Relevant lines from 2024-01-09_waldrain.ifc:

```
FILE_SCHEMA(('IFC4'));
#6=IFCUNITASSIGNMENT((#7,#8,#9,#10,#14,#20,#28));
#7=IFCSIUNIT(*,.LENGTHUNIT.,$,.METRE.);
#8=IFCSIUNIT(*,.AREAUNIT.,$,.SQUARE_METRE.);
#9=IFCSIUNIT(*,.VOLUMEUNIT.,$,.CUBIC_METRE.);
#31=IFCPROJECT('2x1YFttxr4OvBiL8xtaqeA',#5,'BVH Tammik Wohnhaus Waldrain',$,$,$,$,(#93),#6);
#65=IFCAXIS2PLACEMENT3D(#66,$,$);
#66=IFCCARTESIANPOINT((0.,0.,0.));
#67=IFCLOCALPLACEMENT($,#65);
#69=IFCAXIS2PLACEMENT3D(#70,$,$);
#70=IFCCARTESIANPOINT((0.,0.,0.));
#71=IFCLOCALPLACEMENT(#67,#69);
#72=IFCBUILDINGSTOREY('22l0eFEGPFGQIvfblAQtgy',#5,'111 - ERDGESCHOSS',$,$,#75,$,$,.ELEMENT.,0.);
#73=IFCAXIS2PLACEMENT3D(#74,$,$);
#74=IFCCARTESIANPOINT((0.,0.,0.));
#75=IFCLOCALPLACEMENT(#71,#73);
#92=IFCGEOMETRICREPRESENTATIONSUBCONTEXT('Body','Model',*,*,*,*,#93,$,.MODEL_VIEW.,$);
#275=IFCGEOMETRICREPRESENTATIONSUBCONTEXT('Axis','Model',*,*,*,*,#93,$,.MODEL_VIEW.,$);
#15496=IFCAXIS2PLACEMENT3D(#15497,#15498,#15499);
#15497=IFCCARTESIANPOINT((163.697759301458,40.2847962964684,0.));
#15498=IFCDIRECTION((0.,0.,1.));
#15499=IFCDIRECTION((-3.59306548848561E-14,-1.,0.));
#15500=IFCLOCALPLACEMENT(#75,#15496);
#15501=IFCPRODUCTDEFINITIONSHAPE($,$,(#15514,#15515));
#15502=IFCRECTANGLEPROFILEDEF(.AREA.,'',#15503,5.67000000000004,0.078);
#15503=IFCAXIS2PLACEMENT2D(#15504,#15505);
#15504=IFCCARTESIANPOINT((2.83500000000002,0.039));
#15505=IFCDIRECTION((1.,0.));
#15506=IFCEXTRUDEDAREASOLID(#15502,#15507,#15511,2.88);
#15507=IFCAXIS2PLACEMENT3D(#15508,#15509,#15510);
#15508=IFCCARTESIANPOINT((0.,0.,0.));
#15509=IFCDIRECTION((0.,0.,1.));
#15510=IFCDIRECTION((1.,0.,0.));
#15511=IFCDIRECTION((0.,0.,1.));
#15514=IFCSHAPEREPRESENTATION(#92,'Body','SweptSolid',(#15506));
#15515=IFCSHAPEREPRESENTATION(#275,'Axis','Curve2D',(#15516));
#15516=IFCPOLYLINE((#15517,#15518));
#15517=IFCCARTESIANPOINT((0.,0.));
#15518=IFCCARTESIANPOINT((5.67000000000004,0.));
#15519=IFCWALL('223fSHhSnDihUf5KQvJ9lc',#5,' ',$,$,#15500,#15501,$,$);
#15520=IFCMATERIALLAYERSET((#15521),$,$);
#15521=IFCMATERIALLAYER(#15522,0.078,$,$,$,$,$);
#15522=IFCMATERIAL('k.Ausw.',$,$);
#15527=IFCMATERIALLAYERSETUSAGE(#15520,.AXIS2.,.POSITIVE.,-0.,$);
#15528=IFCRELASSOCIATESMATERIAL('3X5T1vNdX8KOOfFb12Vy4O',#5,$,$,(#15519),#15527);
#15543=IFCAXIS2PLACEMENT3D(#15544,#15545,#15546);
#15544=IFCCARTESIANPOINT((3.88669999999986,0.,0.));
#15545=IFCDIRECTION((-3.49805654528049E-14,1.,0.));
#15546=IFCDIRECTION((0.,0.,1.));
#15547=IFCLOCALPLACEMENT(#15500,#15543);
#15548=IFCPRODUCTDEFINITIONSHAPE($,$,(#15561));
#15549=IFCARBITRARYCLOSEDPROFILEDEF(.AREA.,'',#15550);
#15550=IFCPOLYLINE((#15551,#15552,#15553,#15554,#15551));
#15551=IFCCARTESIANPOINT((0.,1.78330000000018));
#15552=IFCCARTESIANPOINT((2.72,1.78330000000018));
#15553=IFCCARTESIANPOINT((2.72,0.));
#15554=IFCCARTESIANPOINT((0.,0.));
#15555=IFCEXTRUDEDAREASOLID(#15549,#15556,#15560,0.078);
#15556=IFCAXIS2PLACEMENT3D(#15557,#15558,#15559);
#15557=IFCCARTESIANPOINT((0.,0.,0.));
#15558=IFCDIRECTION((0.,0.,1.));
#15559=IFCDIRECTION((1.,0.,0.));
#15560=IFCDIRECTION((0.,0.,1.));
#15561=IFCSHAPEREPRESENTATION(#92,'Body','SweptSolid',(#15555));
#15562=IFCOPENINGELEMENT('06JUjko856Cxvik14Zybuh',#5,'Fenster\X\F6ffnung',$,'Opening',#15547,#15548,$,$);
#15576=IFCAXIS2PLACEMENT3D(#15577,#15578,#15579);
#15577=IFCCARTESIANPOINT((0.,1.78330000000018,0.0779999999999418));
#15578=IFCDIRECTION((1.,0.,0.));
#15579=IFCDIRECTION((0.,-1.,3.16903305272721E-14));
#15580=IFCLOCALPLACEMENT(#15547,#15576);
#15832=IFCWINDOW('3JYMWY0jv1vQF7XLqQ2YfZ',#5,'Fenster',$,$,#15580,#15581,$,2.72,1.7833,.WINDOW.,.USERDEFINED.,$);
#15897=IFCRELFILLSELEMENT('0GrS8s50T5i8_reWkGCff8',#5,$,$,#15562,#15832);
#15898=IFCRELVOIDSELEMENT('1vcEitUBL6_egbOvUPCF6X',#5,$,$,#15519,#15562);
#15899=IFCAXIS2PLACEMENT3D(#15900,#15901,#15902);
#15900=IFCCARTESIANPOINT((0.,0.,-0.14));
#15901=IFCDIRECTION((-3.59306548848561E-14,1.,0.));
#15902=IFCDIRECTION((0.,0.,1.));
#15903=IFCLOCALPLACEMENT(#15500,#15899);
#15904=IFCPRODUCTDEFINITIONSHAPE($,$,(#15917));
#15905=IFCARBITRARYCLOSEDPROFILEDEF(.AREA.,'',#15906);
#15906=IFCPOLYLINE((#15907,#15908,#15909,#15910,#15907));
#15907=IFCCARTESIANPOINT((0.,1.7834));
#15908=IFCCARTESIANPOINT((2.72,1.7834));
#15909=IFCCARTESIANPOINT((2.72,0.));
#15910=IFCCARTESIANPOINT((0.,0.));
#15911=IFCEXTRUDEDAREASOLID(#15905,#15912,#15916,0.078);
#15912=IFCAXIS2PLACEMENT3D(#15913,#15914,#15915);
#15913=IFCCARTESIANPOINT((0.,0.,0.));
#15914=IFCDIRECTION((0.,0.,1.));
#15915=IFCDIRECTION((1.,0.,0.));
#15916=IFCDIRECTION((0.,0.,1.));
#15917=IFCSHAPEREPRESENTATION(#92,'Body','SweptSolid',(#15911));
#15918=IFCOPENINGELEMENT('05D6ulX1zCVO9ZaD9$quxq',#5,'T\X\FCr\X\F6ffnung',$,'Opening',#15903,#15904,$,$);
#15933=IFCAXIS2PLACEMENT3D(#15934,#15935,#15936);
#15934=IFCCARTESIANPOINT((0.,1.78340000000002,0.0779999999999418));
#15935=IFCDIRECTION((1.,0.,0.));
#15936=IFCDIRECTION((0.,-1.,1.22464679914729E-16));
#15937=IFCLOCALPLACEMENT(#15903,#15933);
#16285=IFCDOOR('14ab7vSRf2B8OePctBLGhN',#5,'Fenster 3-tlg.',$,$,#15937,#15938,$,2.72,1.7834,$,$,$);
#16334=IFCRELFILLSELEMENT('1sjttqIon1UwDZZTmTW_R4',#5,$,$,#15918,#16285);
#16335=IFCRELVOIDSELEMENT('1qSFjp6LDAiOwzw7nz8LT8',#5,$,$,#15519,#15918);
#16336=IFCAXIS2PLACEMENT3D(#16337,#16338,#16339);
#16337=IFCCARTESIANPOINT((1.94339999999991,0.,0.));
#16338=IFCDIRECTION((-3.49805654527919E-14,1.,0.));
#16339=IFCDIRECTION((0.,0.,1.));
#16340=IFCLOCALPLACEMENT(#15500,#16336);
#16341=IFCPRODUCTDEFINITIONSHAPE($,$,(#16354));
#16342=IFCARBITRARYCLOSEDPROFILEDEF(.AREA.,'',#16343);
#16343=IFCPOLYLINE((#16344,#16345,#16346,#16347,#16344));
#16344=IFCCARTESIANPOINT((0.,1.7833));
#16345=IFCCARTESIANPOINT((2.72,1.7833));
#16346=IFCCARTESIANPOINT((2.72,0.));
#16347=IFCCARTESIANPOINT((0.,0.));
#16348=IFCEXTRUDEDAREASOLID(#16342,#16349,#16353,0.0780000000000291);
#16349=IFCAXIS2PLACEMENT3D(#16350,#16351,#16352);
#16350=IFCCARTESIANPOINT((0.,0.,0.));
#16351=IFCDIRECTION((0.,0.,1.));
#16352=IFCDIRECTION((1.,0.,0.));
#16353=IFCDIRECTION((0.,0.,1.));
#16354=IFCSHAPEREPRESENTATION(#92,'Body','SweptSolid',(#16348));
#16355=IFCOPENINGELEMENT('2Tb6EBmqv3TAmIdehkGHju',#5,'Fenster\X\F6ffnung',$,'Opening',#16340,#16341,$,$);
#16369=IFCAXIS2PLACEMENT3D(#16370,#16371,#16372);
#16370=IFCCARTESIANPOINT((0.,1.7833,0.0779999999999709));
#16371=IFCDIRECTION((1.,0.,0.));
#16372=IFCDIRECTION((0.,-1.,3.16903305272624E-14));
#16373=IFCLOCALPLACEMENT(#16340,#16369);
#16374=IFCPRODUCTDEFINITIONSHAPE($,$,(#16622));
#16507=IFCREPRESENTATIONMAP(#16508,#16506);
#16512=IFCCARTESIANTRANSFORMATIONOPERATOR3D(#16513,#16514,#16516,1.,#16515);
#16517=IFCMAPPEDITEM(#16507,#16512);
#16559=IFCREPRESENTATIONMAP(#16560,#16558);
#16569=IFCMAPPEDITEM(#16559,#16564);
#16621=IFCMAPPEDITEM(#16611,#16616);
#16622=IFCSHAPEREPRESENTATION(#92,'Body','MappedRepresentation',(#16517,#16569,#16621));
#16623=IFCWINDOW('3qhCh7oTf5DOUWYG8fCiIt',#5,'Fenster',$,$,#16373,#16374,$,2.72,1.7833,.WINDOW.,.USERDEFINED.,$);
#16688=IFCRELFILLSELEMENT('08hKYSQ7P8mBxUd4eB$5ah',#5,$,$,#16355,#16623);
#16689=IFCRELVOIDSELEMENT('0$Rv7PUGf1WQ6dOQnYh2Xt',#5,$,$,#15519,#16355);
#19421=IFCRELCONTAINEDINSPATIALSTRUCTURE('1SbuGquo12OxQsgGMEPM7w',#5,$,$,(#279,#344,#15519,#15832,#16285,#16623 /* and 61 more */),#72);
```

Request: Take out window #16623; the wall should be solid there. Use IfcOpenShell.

```python
import ifcopenshell
import ifcopenshell.api.feature
import ifcopenshell.api.root
import ifcopenshell.geom
import ifcopenshell.util.shape

model = ifcopenshell.open("2024-01-09_waldrain.ifc")
settings = ifcopenshell.geom.settings()


def volume(element):
    """Net volume in cubic metres, openings subtracted."""
    shape = ifcopenshell.geom.create_shape(settings, element)
    return ifcopenshell.util.shape.get_volume(shape.geometry)


window = model.by_id(16623)
opening = window.FillsVoids[0].RelatingOpeningElement
wall = opening.VoidsElements[0].RelatingBuildingElement
before = volume(wall)

ifcopenshell.api.root.remove_product(model, product=window)
ifcopenshell.api.feature.remove_feature(model, feature=opening)

after = volume(wall)

print(f"wall volume {before:.3f} -> {after:.3f} m3")

model.write("2024-01-09_waldrain_rev.ifc")
```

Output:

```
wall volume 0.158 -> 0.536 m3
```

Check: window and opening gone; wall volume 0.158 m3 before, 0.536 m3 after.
